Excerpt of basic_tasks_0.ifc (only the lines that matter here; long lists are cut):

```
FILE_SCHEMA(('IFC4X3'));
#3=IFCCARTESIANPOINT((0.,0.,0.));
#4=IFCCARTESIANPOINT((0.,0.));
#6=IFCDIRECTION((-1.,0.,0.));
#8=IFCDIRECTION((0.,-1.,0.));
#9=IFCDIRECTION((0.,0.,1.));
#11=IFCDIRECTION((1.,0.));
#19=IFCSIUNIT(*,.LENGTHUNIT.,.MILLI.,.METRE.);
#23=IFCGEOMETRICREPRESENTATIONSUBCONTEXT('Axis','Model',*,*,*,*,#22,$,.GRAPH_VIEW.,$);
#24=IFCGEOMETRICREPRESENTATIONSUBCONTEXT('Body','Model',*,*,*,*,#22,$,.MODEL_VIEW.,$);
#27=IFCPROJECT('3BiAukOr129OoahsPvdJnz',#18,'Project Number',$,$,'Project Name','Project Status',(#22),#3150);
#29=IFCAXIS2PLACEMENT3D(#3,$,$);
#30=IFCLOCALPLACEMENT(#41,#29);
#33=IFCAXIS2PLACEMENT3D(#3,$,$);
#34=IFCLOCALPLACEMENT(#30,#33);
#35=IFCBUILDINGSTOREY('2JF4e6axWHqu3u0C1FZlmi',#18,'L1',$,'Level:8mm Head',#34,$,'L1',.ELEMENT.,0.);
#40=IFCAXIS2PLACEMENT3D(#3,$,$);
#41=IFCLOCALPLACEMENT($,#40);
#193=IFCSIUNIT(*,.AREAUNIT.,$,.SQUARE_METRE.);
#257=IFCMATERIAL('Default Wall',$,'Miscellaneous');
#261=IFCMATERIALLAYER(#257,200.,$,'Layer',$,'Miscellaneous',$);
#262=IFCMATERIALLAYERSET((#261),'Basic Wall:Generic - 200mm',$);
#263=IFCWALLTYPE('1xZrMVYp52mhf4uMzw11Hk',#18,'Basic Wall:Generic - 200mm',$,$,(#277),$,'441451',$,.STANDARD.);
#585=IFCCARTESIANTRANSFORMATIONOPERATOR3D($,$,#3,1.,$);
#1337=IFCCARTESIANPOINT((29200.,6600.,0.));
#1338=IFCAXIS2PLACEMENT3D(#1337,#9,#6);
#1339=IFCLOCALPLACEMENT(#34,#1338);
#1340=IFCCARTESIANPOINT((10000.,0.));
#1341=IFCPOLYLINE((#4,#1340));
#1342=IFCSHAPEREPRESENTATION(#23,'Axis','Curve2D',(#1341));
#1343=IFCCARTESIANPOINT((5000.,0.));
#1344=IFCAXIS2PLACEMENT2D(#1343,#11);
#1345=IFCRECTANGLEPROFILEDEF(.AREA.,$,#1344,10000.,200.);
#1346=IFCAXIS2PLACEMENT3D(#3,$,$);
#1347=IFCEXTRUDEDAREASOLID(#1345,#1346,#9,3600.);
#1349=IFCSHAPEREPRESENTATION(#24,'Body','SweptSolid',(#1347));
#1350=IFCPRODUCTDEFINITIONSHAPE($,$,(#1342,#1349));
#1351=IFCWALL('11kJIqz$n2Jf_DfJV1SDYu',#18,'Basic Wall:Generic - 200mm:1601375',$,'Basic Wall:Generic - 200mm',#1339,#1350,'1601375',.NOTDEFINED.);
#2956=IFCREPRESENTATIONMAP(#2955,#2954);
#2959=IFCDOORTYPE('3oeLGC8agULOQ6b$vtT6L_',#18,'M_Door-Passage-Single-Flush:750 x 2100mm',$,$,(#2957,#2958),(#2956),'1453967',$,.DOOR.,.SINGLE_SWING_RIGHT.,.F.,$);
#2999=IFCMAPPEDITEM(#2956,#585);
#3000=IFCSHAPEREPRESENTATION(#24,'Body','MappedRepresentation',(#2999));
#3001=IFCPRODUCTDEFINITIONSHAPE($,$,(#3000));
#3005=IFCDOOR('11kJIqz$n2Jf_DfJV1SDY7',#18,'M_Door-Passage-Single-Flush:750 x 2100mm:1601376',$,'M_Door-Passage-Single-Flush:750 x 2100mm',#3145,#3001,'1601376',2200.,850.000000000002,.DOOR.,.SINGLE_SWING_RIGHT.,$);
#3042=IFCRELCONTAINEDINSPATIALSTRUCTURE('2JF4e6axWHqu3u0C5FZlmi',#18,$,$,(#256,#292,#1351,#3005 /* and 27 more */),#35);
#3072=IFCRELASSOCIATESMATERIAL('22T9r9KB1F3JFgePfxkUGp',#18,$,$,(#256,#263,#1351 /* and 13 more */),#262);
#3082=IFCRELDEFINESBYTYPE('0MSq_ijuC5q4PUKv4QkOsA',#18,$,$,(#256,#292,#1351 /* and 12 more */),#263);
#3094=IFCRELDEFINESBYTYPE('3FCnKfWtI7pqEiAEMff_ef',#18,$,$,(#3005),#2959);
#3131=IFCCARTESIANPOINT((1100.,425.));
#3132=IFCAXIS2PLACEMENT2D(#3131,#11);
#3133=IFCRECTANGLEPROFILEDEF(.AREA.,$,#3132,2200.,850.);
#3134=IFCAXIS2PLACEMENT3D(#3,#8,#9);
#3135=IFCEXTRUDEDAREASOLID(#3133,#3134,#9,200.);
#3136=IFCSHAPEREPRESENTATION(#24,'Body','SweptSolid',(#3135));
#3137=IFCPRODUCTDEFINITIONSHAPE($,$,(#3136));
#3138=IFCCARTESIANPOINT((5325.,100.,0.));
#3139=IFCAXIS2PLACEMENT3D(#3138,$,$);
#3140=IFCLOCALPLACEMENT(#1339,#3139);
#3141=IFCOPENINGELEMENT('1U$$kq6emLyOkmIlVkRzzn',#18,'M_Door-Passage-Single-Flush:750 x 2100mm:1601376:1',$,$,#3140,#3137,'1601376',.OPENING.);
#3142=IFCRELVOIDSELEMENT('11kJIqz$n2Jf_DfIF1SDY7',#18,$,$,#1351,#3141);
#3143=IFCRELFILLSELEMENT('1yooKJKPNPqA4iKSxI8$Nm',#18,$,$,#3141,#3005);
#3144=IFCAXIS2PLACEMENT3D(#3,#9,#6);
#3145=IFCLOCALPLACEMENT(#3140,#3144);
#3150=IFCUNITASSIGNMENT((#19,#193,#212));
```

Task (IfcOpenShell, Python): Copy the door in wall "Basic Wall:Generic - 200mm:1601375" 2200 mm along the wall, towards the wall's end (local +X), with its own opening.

```python
import ifcopenshell
import ifcopenshell.api.feature
import ifcopenshell.api.geometry
import ifcopenshell.api.root
import ifcopenshell.geom
import ifcopenshell.util.element
import ifcopenshell.util.placement
import ifcopenshell.util.shape
import ifcopenshell.util.unit

model = ifcopenshell.open("basic_tasks_0.ifc")
unit_scale = ifcopenshell.util.unit.calculate_unit_scale(model)
settings = ifcopenshell.geom.settings()


def volume(element):
    """Net volume in cubic metres, openings subtracted."""
    shape = ifcopenshell.geom.create_shape(settings, element)
    return ifcopenshell.util.shape.get_volume(shape.geometry)


def reuse_history(source, copy):
    """copy_class also copies each property set's owner history, people and application; keep the originals."""
    for rel in copy.IsDefinedBy:
        if rel.is_a("IfcRelDefinesByProperties") and (history := rel.RelatingPropertyDefinition.OwnerHistory):
            rel.RelatingPropertyDefinition.OwnerHistory = source.OwnerHistory
            ifcopenshell.util.element.remove_deep2(model, history)


door = model.by_id(3005)
opening = door.FillsVoids[0].RelatingOpeningElement
wall = opening.VoidsElements[0].RelatingBuildingElement
before = volume(wall)
shift = ifcopenshell.util.placement.get_local_placement(wall.ObjectPlacement)[:3, 0] * 2.2 / unit_scale

# copy_class copies the void relationship, type, container and properties, but no geometry.
new_opening = ifcopenshell.api.root.copy_class(model, product=opening)
new_opening.Representation = ifcopenshell.util.element.copy_deep(
    model, opening.Representation, exclude=["IfcGeometricRepresentationContext", "IfcRepresentationMap"]
)
new_opening.Name = "M_Door-Passage-Single-Flush:750 x 2100mm"
new_opening.Tag = None
new_door = ifcopenshell.api.root.copy_class(model, product=door)
new_door.Representation = ifcopenshell.util.element.copy_deep(
    model, door.Representation, exclude=["IfcGeometricRepresentationContext", "IfcRepresentationMap"]
)
new_door.Name = "M_Door-Passage-Single-Flush:750 x 2100mm"
new_door.Tag = None
reuse_history(door, new_door)
ifcopenshell.api.feature.add_filling(model, opening=new_opening, element=new_door)

for old, new in ((opening, new_opening), (door, new_door)):
    matrix = ifcopenshell.util.placement.get_local_placement(old.ObjectPlacement)
    matrix[:3, 3] += shift
    ifcopenshell.api.geometry.edit_object_placement(model, product=new, matrix=matrix, is_si=False)

after = volume(wall)

print(f"wall volume {before:.3f} -> {after:.3f} m3")

model.write("basic_tasks_0_updated.ifc")
```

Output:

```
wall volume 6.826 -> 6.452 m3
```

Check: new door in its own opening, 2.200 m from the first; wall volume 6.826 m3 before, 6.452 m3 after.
